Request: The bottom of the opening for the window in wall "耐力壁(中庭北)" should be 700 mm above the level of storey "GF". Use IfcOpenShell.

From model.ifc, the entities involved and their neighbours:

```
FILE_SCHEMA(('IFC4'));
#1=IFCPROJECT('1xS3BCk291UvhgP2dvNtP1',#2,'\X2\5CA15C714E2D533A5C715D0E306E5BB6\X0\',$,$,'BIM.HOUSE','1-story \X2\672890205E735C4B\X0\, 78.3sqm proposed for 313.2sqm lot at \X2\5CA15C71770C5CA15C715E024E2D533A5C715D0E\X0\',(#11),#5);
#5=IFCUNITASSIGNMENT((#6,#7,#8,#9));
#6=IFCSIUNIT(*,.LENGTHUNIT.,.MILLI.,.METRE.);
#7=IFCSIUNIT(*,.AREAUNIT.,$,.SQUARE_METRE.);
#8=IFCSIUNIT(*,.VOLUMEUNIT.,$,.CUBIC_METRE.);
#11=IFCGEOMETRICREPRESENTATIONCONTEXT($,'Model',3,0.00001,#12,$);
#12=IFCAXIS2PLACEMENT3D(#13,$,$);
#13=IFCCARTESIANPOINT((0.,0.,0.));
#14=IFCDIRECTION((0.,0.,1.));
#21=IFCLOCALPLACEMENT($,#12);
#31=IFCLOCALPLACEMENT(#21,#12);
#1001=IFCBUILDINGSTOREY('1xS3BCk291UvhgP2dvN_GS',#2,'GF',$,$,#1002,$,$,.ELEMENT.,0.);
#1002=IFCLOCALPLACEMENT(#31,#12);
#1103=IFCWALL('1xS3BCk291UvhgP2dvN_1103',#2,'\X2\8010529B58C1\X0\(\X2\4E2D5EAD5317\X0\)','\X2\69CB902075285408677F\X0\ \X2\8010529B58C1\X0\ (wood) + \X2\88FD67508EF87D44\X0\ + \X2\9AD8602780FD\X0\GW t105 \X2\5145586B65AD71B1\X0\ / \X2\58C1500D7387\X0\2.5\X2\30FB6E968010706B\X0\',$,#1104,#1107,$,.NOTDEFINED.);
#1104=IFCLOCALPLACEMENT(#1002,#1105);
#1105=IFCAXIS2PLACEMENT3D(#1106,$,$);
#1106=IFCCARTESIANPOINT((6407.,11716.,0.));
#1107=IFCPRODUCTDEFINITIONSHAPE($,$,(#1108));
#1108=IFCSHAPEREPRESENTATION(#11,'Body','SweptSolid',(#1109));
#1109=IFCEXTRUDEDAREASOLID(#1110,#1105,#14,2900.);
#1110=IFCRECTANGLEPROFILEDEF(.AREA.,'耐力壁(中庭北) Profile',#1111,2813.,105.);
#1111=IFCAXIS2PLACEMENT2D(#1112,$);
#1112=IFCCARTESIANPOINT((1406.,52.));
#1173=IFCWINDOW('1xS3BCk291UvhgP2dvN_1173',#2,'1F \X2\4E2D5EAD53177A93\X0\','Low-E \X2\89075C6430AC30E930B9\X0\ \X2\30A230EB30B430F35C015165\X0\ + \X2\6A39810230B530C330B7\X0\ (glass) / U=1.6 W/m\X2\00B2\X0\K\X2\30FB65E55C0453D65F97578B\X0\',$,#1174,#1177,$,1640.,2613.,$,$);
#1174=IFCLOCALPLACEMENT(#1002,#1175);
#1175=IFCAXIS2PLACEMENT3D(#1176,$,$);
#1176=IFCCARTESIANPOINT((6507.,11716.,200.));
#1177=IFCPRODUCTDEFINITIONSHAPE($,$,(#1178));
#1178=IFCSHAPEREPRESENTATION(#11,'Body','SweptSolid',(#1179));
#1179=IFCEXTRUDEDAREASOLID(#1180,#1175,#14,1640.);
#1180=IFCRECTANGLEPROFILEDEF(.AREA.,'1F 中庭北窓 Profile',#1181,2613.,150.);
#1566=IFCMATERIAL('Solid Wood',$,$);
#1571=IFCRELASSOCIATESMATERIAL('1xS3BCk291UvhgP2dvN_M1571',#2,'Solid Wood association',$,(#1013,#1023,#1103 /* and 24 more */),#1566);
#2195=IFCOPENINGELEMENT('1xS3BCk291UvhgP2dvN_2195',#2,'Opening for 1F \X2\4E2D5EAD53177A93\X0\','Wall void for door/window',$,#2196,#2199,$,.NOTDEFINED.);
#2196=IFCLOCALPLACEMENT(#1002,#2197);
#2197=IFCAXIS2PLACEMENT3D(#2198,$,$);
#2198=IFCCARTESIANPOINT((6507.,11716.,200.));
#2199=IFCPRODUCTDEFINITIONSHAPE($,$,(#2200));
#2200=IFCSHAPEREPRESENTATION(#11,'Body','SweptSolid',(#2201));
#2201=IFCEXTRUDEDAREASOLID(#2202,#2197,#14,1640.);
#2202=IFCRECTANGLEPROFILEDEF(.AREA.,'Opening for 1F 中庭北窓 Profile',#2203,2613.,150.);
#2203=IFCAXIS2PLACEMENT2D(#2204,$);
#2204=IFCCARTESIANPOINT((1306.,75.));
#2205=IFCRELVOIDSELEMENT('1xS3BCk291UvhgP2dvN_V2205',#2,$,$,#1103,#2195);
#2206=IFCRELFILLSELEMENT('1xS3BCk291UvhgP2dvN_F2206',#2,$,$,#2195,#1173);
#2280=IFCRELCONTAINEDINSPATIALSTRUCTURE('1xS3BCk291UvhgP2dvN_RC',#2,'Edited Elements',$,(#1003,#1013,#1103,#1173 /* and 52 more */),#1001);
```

```python
import numpy as np
import ifcopenshell
import ifcopenshell.api.geometry
import ifcopenshell.geom
import ifcopenshell.util.element
import ifcopenshell.util.placement
import ifcopenshell.util.shape
import ifcopenshell.util.unit

model = ifcopenshell.open("model.ifc")
unit_scale = ifcopenshell.util.unit.calculate_unit_scale(model)

window = model.by_guid("1xS3BCk291UvhgP2dvN_1173")
opening = window.FillsVoids[0].RelatingOpeningElement
storey = ifcopenshell.util.element.get_container(window, ifc_class="IfcBuildingStorey")
level = ifcopenshell.util.placement.get_local_placement(storey.ObjectPlacement)[2, 3]

# The opening's origin need not be at the sill, so measure its lowest point.
shape = ifcopenshell.geom.create_shape(ifcopenshell.geom.settings(), opening)
bottom = ifcopenshell.util.shape.get_shape_bottom_elevation(shape, shape.geometry) / unit_scale
dz = level + 0.7 / unit_scale - bottom

shift = np.array([0.0, 0.0, dz])
# The window is not placed relative to its opening, so move both.
for product in (opening, window):
    matrix = ifcopenshell.util.placement.get_local_placement(product.ObjectPlacement)
    matrix[:3, 3] += shift
    ifcopenshell.api.geometry.edit_object_placement(model, product=product, matrix=matrix, is_si=False)

print(f"moved by {dz * unit_scale:+.3f} m")

model.write("model_updated.ifc")
```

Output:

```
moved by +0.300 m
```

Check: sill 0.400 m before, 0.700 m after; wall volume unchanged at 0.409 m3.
